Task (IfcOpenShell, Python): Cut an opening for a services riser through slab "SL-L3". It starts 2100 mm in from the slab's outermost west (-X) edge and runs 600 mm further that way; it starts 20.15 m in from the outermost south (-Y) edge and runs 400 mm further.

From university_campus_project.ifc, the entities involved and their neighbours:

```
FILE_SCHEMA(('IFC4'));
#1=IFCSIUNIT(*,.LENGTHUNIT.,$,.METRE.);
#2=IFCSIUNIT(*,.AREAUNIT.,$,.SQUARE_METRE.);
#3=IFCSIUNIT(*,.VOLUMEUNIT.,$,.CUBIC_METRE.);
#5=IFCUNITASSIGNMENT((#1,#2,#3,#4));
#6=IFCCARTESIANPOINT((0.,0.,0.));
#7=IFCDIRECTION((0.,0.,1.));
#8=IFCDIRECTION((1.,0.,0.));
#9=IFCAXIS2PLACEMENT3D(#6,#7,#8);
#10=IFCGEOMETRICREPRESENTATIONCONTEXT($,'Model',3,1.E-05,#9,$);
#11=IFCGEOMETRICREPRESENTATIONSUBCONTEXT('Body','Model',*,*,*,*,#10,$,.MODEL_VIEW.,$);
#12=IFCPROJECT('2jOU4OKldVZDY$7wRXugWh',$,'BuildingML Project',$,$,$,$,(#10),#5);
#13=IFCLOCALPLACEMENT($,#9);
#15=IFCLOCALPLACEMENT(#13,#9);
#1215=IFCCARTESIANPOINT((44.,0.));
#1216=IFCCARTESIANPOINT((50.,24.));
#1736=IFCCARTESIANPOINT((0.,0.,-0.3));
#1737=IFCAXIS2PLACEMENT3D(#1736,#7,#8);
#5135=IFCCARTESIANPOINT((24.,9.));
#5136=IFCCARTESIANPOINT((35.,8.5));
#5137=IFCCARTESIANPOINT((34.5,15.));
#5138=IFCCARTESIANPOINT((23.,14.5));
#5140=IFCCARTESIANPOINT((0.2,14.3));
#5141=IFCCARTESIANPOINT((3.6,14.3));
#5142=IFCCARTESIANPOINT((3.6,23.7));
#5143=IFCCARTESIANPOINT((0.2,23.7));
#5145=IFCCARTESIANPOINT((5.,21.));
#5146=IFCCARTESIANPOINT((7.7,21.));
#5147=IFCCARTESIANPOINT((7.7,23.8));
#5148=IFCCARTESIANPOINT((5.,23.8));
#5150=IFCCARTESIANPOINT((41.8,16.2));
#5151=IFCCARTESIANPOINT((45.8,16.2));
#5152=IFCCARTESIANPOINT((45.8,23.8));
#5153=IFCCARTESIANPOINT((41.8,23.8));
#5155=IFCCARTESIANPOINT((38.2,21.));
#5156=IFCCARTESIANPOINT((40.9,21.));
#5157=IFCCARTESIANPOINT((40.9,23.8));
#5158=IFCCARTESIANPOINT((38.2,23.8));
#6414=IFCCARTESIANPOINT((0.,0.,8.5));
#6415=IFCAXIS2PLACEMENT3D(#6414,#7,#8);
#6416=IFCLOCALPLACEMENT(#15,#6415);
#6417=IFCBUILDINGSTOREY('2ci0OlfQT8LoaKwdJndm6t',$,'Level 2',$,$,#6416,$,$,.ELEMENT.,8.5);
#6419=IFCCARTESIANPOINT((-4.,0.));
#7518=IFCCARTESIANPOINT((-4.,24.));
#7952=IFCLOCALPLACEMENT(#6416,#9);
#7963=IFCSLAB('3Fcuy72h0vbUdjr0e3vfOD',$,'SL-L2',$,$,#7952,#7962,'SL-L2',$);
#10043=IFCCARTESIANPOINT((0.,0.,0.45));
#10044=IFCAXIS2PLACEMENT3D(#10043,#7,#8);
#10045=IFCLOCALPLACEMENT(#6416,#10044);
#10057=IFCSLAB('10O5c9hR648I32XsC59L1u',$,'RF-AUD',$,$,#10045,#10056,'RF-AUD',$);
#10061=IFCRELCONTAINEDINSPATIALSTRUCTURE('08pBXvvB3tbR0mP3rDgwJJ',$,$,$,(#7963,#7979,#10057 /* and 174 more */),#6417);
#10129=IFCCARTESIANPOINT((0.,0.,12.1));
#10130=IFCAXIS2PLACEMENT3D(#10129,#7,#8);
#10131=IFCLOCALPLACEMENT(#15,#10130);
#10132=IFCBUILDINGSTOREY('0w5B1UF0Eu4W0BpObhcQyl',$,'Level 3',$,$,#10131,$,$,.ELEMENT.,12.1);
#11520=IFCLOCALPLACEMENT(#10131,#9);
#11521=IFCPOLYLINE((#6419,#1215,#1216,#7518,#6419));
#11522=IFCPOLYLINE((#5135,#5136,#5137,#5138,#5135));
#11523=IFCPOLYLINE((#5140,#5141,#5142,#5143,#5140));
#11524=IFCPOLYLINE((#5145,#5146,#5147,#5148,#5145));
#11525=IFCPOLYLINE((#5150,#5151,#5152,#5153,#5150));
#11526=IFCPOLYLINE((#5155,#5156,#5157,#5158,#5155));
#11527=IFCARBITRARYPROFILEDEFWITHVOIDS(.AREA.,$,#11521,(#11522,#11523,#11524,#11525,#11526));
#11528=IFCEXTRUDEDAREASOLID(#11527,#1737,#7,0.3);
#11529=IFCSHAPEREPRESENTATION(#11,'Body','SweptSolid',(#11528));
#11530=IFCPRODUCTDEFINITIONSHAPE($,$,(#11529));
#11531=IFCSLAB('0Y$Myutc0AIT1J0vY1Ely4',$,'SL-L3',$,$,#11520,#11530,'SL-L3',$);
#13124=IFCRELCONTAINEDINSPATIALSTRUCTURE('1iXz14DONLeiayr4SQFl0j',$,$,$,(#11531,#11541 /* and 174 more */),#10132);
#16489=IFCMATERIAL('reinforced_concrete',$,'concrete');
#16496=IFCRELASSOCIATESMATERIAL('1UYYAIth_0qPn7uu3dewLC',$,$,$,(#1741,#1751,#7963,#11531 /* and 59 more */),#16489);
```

```python
import numpy as np
import ifcopenshell
import ifcopenshell.api.feature
import ifcopenshell.api.geometry
import ifcopenshell.api.root
import ifcopenshell.geom
import ifcopenshell.util.placement
import ifcopenshell.util.representation
import ifcopenshell.util.shape
import ifcopenshell.util.unit

model = ifcopenshell.open("university_campus_project.ifc")
unit_scale = ifcopenshell.util.unit.calculate_unit_scale(model)
settings = ifcopenshell.geom.settings()


def volume(element):
    """Net volume in cubic metres, openings subtracted."""
    shape = ifcopenshell.geom.create_shape(settings, element)
    return ifcopenshell.util.shape.get_volume(shape.geometry)


slab = model.by_guid("0Y$Myutc0AIT1J0vY1Ely4")
before = volume(slab)

# Extent in the slab's own axes, in metres. The edges named are its -X and -Y sides.
slab_shape = ifcopenshell.geom.create_shape(settings, slab)
vertices = ifcopenshell.util.shape.get_vertices(slab_shape.geometry)
x_min, y_min, bottom = vertices.min(axis=0)
top = vertices[:, 2].max()

opening = ifcopenshell.api.root.create_entity(model, ifc_class="IfcOpeningElement", name="Services riser opening", predefined_type="OPENING")
context = ifcopenshell.util.representation.get_context(model, "Model", "Body", "MODEL_VIEW")
width, depth = 0.6, 0.4
outline = [(0.0, 0.0), (width, 0.0), (width, depth), (0.0, depth), (0.0, 0.0)]
# Overshoot both faces by 50 mm so the cut is clean.
shape = ifcopenshell.api.geometry.add_slab_representation(
    model, context=context, depth=top - bottom + 0.1, polyline=outline
)
ifcopenshell.api.geometry.assign_representation(model, product=opening, representation=shape)

matrix = ifcopenshell.util.placement.get_local_placement(slab.ObjectPlacement)
matrix[:, 3] = matrix @ np.append(np.array([x_min + 2.1, y_min + 20.15, bottom - 0.05]) / unit_scale, 1.0)
ifcopenshell.api.geometry.edit_object_placement(model, product=opening, matrix=matrix, is_si=False)
ifcopenshell.api.feature.add_feature(model, feature=opening, element=slab)

after = volume(slab)

print(f"slab volume {before:.3f} -> {after:.3f} m3")

model.write("university_campus_project_rev.ifc")
```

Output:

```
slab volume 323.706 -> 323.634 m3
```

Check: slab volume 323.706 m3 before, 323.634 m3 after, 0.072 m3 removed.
